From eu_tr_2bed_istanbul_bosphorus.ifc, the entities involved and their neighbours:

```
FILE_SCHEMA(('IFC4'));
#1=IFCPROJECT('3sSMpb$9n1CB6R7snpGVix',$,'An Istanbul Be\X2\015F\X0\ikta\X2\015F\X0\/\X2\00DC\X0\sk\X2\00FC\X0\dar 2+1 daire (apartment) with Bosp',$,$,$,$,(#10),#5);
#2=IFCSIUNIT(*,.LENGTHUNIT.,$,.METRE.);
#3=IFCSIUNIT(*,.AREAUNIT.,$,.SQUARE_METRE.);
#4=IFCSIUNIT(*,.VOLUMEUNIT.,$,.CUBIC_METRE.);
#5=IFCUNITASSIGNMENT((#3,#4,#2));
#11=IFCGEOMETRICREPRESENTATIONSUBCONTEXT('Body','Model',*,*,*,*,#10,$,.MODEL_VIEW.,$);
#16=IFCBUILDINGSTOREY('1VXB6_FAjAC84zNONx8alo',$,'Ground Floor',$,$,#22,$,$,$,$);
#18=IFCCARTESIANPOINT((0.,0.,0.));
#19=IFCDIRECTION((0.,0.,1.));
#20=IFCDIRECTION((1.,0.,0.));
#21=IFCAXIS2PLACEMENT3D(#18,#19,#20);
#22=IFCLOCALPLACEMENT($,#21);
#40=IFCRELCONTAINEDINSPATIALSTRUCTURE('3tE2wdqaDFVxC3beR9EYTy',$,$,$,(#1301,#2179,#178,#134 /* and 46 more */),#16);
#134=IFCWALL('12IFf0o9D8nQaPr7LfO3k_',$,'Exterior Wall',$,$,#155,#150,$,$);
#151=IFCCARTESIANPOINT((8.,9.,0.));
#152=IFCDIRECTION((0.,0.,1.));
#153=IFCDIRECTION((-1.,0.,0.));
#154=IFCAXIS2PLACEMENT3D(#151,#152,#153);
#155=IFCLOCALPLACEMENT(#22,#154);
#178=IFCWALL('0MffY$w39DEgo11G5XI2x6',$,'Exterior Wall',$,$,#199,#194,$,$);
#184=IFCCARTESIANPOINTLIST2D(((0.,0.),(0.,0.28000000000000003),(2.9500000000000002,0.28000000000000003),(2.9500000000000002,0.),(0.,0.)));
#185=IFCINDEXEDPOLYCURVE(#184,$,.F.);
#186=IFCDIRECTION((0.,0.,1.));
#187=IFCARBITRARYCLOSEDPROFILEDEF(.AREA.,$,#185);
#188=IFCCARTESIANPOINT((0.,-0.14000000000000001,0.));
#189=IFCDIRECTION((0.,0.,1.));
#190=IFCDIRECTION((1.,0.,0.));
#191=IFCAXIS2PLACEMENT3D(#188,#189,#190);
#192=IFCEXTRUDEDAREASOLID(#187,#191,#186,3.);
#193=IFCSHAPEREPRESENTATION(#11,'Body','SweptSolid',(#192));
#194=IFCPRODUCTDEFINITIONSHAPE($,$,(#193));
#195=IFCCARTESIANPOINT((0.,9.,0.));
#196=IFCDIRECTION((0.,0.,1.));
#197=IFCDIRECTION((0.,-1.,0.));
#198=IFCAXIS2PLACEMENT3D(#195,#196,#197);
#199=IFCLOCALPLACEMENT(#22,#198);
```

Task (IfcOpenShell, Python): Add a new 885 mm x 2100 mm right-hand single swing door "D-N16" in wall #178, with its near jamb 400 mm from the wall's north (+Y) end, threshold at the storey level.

```python
import numpy as np
import ifcopenshell
import ifcopenshell.api.feature
import ifcopenshell.api.geometry
import ifcopenshell.api.root
import ifcopenshell.api.spatial
import ifcopenshell.geom
import ifcopenshell.util.element
import ifcopenshell.util.placement
import ifcopenshell.util.representation
import ifcopenshell.util.shape
import ifcopenshell.util.unit

model = ifcopenshell.open("eu_tr_2bed_istanbul_bosphorus.ifc")
unit_scale = ifcopenshell.util.unit.calculate_unit_scale(model)
settings = ifcopenshell.geom.settings()


def volume(element):
    """Net volume in cubic metres, openings subtracted."""
    shape = ifcopenshell.geom.create_shape(settings, element)
    return ifcopenshell.util.shape.get_volume(shape.geometry)


wall = model.by_guid("0MffY$w39DEgo11G5XI2x6")
storey = ifcopenshell.util.element.get_container(wall, ifc_class="IfcBuildingStorey")
context = ifcopenshell.util.representation.get_context(model, "Model", "Body", "MODEL_VIEW")
before = volume(wall)

width, height, from_end, sill = 0.885, 2.1, 0.4, 0.0  # metres

# The wall runs along its own X axis, and the end named is its -X end.
wall_shape = ifcopenshell.geom.create_shape(settings, wall)
x, y, z = ifcopenshell.util.shape.get_vertices(wall_shape.geometry).T
start = x.min() + from_end
face, thickness = float(y.min()), float(y.max() - y.min())
wall_matrix = ifcopenshell.util.placement.get_local_placement(wall.ObjectPlacement)
level = ifcopenshell.util.placement.get_local_placement(storey.ObjectPlacement)[2, 3]


def in_wall(x, y):
    """Placement at x, y metres in the wall's axes, at sill height."""
    matrix = wall_matrix.copy()
    matrix[:, 3] = wall_matrix @ np.array([x / unit_scale, y / unit_scale, 0.0, 1.0])
    matrix[2, 3] = level + sill / unit_scale
    return matrix


# Opening: a box that overshoots both wall faces by 50 mm.
opening = ifcopenshell.api.root.create_entity(model, ifc_class="IfcOpeningElement", predefined_type="OPENING")
box = ifcopenshell.api.geometry.add_wall_representation(
    model, context=context, length=width, height=height, thickness=thickness + 0.1
)
ifcopenshell.api.geometry.assign_representation(model, product=opening, representation=box)
ifcopenshell.api.geometry.edit_object_placement(model, product=opening, matrix=in_wall(start, face - 0.05), is_si=False)
ifcopenshell.api.feature.add_feature(model, feature=opening, element=wall)

door = ifcopenshell.api.root.create_entity(model, ifc_class="IfcDoor", name="D-N16", predefined_type="DOOR")
door.OverallWidth, door.OverallHeight = width / unit_scale, height / unit_scale
door.OperationType = "SINGLE_SWING_RIGHT"
body = ifcopenshell.api.geometry.add_door_representation(
    model,
    context=context,
    overall_width=door.OverallWidth,
    overall_height=door.OverallHeight,
    operation_type="SINGLE_SWING_RIGHT",
    lining_properties={"LiningDepth": thickness / unit_scale, "ThresholdDepth": thickness / unit_scale},
)
ifcopenshell.api.geometry.assign_representation(model, product=door, representation=body)
ifcopenshell.api.spatial.assign_container(model, products=[door], relating_structure=storey)
ifcopenshell.api.feature.add_filling(model, opening=opening, element=door)

# The lining spans the wall, so the door starts at the wall face.
ifcopenshell.api.geometry.edit_object_placement(model, product=door, matrix=in_wall(start, face), is_si=False)

after = volume(wall)

print(f"wall volume {before:.3f} -> {after:.3f} m3")

model.write("eu_tr_2bed_istanbul_bosphorus_v2.ifc")
```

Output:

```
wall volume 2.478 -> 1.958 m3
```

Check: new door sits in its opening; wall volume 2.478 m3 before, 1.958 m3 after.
